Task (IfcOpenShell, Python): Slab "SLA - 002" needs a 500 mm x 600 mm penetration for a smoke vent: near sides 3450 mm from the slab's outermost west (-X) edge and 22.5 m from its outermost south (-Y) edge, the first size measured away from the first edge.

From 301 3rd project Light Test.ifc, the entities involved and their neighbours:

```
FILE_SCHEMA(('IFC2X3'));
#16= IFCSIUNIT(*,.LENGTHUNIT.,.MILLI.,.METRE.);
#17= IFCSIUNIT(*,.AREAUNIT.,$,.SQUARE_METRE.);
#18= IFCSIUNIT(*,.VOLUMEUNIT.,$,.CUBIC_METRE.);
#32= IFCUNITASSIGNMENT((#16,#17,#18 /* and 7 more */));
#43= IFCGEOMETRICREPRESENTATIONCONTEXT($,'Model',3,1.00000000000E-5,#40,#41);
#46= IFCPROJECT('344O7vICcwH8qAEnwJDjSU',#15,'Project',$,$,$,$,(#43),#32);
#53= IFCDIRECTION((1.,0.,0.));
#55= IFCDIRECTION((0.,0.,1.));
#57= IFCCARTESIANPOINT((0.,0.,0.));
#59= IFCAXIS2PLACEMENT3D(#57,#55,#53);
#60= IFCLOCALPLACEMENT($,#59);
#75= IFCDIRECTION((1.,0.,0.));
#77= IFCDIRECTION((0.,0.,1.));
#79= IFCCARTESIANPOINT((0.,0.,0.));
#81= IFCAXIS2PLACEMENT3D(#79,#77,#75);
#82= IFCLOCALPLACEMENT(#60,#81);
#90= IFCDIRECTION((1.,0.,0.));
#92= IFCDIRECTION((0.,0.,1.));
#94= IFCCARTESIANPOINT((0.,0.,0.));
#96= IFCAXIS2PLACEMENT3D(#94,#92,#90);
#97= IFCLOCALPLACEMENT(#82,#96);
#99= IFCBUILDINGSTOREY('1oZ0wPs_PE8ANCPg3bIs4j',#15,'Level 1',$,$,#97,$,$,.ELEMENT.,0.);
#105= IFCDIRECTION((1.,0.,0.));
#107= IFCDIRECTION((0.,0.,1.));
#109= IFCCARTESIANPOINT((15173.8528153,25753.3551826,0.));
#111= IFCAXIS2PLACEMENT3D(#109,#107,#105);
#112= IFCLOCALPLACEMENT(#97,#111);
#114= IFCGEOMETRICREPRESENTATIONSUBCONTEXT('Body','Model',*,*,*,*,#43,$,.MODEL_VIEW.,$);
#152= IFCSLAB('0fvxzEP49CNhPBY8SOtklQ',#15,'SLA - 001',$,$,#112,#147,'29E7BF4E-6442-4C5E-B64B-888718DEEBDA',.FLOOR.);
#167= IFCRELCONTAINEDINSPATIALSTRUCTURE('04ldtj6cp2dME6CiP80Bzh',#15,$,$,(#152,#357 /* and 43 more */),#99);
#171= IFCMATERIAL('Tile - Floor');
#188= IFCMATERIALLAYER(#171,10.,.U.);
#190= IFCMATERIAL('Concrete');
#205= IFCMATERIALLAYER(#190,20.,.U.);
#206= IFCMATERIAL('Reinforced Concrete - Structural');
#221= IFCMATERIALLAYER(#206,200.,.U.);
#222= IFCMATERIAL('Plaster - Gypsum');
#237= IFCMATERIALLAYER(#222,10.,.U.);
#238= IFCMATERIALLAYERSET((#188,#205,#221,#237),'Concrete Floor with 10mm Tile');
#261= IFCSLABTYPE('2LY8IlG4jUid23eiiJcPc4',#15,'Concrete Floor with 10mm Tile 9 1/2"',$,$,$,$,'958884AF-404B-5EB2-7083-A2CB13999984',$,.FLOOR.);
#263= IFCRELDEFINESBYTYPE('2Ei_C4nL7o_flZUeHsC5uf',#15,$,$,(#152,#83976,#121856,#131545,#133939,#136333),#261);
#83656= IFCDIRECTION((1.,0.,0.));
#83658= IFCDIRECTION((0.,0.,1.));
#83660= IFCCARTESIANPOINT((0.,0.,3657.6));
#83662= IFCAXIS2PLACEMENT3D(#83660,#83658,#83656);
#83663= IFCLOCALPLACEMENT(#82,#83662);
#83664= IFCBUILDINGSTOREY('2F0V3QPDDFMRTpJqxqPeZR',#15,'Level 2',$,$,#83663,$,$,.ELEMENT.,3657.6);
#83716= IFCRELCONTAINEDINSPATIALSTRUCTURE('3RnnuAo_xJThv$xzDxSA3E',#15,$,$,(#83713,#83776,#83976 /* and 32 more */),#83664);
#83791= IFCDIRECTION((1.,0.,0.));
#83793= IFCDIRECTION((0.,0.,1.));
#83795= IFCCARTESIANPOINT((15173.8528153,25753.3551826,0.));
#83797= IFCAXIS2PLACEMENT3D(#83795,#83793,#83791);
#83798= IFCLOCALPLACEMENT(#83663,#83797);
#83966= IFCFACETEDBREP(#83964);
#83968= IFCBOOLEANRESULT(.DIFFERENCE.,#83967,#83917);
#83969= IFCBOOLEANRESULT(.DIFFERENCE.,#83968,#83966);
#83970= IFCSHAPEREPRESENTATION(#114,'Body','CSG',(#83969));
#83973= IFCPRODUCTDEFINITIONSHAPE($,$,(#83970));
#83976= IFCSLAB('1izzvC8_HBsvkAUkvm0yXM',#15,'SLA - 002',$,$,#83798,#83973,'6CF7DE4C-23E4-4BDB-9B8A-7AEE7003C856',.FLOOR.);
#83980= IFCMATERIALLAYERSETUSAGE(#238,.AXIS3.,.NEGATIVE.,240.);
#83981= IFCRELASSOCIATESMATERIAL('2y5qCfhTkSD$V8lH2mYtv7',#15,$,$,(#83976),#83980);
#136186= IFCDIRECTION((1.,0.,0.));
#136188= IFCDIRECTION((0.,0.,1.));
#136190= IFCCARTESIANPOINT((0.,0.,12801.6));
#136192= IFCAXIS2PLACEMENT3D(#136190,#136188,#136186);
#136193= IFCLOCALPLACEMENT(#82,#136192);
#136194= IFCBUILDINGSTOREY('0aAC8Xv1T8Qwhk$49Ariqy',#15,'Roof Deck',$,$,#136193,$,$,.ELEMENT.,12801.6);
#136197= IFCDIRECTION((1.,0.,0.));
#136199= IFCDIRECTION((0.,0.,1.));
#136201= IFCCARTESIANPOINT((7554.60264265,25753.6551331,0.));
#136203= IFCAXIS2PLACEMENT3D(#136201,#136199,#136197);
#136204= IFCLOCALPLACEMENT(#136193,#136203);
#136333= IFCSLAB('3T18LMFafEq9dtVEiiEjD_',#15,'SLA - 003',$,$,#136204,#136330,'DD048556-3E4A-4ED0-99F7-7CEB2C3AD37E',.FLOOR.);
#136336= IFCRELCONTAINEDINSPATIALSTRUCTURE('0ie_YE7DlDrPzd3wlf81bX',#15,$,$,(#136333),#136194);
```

```python
import numpy as np
import ifcopenshell
import ifcopenshell.api.feature
import ifcopenshell.api.geometry
import ifcopenshell.api.root
import ifcopenshell.geom
import ifcopenshell.util.placement
import ifcopenshell.util.representation
import ifcopenshell.util.shape
import ifcopenshell.util.unit

model = ifcopenshell.open("301 3rd project Light Test.ifc")
unit_scale = ifcopenshell.util.unit.calculate_unit_scale(model)
settings = ifcopenshell.geom.settings()


def volume(element):
    """Net volume in cubic metres, openings subtracted."""
    shape = ifcopenshell.geom.create_shape(settings, element)
    return ifcopenshell.util.shape.get_volume(shape.geometry)


slab = model.by_id(83976)
before = volume(slab)

# Extent in the slab's own axes, in metres. The edges named are its -X and -Y sides.
slab_shape = ifcopenshell.geom.create_shape(settings, slab)
vertices = ifcopenshell.util.shape.get_vertices(slab_shape.geometry)
x_min, y_min, bottom = vertices.min(axis=0)
top = vertices[:, 2].max()

opening = ifcopenshell.api.root.create_entity(model, ifc_class="IfcOpeningElement", name="Smoke vent opening")
context = ifcopenshell.util.representation.get_context(model, "Model", "Body", "MODEL_VIEW")
width, depth = 0.5, 0.6
outline = [(0.0, 0.0), (width, 0.0), (width, depth), (0.0, depth), (0.0, 0.0)]
# Overshoot both faces by 50 mm so the cut is clean.
shape = ifcopenshell.api.geometry.add_slab_representation(
    model, context=context, depth=top - bottom + 0.1, polyline=outline
)
ifcopenshell.api.geometry.assign_representation(model, product=opening, representation=shape)

matrix = ifcopenshell.util.placement.get_local_placement(slab.ObjectPlacement)
matrix[:, 3] = matrix @ np.append(np.array([x_min + 3.45, y_min + 22.5, bottom - 0.05]) / unit_scale, 1.0)
ifcopenshell.api.geometry.edit_object_placement(model, product=opening, matrix=matrix, is_si=False)
ifcopenshell.api.feature.add_feature(model, feature=opening, element=slab)

after = volume(slab)

print(f"slab volume {before:.3f} -> {after:.3f} m3")

model.write("301 3rd project Light Test_v2.ifc")
```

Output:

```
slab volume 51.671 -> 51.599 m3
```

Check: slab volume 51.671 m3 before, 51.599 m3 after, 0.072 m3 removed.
